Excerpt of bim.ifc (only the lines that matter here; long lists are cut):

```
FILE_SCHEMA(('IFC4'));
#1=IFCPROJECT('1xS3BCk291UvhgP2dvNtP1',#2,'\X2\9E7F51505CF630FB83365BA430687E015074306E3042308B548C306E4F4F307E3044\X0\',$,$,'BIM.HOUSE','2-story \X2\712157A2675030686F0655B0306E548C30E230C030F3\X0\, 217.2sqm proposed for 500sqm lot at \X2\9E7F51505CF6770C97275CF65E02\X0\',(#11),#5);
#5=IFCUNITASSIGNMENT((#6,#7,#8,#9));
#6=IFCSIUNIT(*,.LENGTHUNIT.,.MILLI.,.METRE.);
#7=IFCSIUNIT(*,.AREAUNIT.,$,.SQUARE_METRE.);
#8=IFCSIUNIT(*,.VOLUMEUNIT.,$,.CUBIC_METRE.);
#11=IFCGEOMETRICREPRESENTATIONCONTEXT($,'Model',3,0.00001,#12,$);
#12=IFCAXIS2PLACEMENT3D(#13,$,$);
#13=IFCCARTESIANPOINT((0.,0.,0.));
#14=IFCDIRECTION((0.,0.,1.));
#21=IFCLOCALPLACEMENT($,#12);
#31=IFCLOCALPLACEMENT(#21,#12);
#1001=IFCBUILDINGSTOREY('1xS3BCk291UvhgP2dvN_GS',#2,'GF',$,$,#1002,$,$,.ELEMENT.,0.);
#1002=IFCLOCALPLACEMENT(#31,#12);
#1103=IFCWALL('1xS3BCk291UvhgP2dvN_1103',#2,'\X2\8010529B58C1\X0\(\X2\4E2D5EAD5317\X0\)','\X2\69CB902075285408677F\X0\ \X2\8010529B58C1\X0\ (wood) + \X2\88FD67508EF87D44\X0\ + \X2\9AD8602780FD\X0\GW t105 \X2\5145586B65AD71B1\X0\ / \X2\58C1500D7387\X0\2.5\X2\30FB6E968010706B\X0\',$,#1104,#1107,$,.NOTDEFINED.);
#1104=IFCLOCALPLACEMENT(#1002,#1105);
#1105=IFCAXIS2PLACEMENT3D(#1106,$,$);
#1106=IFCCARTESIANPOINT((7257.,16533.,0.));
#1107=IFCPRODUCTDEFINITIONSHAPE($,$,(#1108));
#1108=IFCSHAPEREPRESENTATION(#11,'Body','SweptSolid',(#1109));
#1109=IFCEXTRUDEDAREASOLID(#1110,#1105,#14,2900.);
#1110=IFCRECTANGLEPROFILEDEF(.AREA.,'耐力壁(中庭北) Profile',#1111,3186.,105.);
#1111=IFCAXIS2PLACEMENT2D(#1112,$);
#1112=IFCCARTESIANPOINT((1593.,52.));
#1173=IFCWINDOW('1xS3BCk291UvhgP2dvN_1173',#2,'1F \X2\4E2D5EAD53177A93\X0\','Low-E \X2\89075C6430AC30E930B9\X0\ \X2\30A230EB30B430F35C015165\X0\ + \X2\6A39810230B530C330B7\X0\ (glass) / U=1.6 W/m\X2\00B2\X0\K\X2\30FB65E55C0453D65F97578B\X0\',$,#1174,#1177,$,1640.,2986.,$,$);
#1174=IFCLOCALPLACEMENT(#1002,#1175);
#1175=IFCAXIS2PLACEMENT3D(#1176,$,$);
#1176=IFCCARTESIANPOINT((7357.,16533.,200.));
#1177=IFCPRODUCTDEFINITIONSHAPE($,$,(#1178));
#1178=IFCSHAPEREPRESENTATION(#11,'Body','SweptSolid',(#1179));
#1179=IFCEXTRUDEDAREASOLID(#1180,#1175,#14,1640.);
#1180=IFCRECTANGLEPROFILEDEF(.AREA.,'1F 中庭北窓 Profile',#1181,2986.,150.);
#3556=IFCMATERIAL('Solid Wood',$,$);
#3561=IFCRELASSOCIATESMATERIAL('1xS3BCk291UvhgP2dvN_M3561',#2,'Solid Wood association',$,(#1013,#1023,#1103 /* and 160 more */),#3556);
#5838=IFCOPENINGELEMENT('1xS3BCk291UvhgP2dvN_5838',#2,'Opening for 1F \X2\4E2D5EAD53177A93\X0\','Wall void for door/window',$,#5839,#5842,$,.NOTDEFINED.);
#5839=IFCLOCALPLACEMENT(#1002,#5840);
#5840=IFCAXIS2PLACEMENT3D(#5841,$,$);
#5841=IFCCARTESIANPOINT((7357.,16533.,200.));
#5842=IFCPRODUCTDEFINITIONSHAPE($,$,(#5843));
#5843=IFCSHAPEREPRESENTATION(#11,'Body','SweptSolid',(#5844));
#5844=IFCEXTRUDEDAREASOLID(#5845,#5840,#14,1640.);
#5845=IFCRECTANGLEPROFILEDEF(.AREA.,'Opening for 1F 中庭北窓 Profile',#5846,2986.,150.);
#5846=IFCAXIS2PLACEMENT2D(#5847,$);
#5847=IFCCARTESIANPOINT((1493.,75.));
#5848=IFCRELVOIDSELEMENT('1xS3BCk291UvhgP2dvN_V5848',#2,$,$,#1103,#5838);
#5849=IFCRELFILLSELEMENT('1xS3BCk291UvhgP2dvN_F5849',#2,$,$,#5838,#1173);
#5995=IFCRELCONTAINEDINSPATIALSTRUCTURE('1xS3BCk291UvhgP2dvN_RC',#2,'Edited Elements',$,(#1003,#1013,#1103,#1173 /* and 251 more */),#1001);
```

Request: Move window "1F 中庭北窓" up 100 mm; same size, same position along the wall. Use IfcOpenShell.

```python
import numpy as np
import ifcopenshell
import ifcopenshell.api.geometry
import ifcopenshell.util.placement
import ifcopenshell.util.unit

model = ifcopenshell.open("bim.ifc")
unit_scale = ifcopenshell.util.unit.calculate_unit_scale(model)

window = model.by_guid("1xS3BCk291UvhgP2dvN_1173")
opening = window.FillsVoids[0].RelatingOpeningElement
dz = 100.0

shift = np.array([0.0, 0.0, dz])
# The window is not placed relative to its opening, so move both.
for product in (opening, window):
    matrix = ifcopenshell.util.placement.get_local_placement(product.ObjectPlacement)
    matrix[:3, 3] += shift
    ifcopenshell.api.geometry.edit_object_placement(model, product=product, matrix=matrix, is_si=False)

print(f"moved by {dz * unit_scale:+.3f} m")

model.write("bim_v2.ifc")
```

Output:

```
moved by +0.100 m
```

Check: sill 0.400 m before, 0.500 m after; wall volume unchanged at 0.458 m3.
